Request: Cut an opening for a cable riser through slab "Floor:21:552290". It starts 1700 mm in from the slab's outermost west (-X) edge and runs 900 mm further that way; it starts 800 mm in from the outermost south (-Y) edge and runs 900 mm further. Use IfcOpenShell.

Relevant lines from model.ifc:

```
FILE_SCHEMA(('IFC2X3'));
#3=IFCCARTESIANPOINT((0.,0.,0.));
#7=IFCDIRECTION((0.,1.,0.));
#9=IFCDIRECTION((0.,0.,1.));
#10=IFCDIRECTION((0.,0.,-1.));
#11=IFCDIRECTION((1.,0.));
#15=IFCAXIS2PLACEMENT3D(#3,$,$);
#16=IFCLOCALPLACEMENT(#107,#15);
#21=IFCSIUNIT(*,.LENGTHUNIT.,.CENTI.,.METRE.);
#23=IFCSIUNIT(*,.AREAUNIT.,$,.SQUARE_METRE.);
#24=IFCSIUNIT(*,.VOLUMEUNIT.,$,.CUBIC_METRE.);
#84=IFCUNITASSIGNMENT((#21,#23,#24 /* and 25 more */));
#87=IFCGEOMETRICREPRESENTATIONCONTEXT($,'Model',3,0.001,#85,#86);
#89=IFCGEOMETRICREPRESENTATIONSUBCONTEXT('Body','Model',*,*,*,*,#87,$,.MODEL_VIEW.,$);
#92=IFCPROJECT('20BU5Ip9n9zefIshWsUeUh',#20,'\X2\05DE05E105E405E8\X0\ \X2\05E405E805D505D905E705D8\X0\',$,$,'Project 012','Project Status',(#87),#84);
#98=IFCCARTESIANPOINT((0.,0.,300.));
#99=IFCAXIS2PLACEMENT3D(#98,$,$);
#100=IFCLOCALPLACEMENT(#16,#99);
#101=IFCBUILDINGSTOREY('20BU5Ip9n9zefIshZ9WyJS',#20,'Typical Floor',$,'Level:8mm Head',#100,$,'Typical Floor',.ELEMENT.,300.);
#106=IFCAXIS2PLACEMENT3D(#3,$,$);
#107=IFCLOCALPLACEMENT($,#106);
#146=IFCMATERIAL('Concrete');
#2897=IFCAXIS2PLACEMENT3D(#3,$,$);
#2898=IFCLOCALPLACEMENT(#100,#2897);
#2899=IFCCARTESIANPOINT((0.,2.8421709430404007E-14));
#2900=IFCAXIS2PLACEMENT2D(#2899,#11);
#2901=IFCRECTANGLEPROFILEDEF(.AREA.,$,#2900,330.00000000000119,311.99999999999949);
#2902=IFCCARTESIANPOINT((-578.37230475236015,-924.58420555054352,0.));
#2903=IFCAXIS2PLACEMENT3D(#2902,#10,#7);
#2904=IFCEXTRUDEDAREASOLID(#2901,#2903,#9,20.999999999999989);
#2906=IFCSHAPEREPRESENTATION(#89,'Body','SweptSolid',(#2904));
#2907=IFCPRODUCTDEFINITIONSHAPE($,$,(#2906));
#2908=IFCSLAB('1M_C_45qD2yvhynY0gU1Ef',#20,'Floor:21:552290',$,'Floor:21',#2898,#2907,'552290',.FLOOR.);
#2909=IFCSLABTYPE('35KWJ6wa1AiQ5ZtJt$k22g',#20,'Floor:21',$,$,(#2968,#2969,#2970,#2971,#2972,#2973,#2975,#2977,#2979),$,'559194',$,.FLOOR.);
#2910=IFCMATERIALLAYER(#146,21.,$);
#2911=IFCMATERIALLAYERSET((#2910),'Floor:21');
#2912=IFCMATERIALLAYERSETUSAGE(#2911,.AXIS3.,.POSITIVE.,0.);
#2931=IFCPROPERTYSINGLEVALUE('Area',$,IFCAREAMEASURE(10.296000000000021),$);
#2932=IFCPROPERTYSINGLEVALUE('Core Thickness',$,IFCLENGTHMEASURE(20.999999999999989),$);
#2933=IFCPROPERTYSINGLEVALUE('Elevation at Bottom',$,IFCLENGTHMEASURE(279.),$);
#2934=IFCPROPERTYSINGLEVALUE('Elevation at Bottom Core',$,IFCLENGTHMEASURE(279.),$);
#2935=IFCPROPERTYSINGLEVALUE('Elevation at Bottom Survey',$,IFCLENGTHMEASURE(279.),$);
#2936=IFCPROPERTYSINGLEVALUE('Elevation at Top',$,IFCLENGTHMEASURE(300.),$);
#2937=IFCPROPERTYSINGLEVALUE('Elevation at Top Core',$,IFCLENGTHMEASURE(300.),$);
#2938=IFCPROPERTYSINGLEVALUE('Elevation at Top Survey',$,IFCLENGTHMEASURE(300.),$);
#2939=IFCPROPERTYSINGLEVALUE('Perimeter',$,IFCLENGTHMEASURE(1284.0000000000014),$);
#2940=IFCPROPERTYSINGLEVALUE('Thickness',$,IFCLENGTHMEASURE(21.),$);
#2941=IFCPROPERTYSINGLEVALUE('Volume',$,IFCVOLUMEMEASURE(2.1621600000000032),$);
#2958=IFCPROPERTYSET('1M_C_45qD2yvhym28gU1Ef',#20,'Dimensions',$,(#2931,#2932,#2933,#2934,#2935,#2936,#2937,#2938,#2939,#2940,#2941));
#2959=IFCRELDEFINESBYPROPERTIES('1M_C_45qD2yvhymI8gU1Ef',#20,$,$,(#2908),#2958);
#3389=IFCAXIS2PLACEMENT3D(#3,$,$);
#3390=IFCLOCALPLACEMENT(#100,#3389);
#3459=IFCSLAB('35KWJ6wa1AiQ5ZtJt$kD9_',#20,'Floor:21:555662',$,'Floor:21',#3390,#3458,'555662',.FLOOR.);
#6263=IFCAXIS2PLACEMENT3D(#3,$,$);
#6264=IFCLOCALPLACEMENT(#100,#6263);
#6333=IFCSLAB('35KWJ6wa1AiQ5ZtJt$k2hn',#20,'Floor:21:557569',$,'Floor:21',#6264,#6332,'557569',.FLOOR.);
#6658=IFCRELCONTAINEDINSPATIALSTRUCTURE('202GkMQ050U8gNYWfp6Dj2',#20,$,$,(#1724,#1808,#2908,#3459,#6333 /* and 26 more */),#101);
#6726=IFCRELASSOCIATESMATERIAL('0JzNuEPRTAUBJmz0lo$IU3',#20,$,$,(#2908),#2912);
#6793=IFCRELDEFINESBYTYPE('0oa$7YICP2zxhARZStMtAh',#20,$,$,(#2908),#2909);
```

```python
import numpy as np
import ifcopenshell
import ifcopenshell.api.feature
import ifcopenshell.api.geometry
import ifcopenshell.api.pset
import ifcopenshell.api.root
import ifcopenshell.geom
import ifcopenshell.util.element
import ifcopenshell.util.placement
import ifcopenshell.util.representation
import ifcopenshell.util.shape
import ifcopenshell.util.unit

model = ifcopenshell.open("model.ifc")
unit_scale = ifcopenshell.util.unit.calculate_unit_scale(model)
area_scale = ifcopenshell.util.unit.calculate_unit_scale(model, "AREAUNIT")
volume_scale = ifcopenshell.util.unit.calculate_unit_scale(model, "VOLUMEUNIT")
settings = ifcopenshell.geom.settings()


def volume(element):
    """Net volume in cubic metres, openings subtracted."""
    shape = ifcopenshell.geom.create_shape(settings, element)
    return ifcopenshell.util.shape.get_volume(shape.geometry)


slab = model.by_guid("1M_C_45qD2yvhynY0gU1Ef")
before = volume(slab)

# Extent in the slab's own axes, in metres. The edges named are its -X and -Y sides.
slab_shape = ifcopenshell.geom.create_shape(settings, slab)
vertices = ifcopenshell.util.shape.get_vertices(slab_shape.geometry)
x_min, y_min, bottom = vertices.min(axis=0)
top = vertices[:, 2].max()

opening = ifcopenshell.api.root.create_entity(model, ifc_class="IfcOpeningElement", name="Cable riser opening")
context = ifcopenshell.util.representation.get_context(model, "Model", "Body", "MODEL_VIEW")
width, depth = 0.9, 0.9
outline = [(0.0, 0.0), (width, 0.0), (width, depth), (0.0, depth), (0.0, 0.0)]
# Overshoot both faces by 50 mm so the cut is clean.
shape = ifcopenshell.api.geometry.add_slab_representation(
    model, context=context, depth=top - bottom + 0.1, polyline=outline
)
ifcopenshell.api.geometry.assign_representation(model, product=opening, representation=shape)

matrix = ifcopenshell.util.placement.get_local_placement(slab.ObjectPlacement)
matrix[:, 3] = matrix @ np.append(np.array([x_min + 1.7, y_min + 0.8, bottom - 0.05]) / unit_scale, 1.0)
ifcopenshell.api.geometry.edit_object_placement(model, product=opening, matrix=matrix, is_si=False)
ifcopenshell.api.feature.add_feature(model, feature=opening, element=slab)

after = volume(slab)

# Update the slab's stored quantities.
pset = model.by_id(ifcopenshell.util.element.get_pset(slab, "Dimensions", should_inherit=False)["id"])
ifcopenshell.api.pset.edit_pset(model, pset=pset, properties={
    "Area": model.create_entity("IfcAreaMeasure", after / (top - bottom) / area_scale),
    "Volume": model.create_entity("IfcVolumeMeasure", after / volume_scale),
})

print(f"slab volume {before:.3f} -> {after:.3f} m3")

model.write("model-out.ifc")
```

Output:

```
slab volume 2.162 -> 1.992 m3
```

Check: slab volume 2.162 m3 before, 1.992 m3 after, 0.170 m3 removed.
